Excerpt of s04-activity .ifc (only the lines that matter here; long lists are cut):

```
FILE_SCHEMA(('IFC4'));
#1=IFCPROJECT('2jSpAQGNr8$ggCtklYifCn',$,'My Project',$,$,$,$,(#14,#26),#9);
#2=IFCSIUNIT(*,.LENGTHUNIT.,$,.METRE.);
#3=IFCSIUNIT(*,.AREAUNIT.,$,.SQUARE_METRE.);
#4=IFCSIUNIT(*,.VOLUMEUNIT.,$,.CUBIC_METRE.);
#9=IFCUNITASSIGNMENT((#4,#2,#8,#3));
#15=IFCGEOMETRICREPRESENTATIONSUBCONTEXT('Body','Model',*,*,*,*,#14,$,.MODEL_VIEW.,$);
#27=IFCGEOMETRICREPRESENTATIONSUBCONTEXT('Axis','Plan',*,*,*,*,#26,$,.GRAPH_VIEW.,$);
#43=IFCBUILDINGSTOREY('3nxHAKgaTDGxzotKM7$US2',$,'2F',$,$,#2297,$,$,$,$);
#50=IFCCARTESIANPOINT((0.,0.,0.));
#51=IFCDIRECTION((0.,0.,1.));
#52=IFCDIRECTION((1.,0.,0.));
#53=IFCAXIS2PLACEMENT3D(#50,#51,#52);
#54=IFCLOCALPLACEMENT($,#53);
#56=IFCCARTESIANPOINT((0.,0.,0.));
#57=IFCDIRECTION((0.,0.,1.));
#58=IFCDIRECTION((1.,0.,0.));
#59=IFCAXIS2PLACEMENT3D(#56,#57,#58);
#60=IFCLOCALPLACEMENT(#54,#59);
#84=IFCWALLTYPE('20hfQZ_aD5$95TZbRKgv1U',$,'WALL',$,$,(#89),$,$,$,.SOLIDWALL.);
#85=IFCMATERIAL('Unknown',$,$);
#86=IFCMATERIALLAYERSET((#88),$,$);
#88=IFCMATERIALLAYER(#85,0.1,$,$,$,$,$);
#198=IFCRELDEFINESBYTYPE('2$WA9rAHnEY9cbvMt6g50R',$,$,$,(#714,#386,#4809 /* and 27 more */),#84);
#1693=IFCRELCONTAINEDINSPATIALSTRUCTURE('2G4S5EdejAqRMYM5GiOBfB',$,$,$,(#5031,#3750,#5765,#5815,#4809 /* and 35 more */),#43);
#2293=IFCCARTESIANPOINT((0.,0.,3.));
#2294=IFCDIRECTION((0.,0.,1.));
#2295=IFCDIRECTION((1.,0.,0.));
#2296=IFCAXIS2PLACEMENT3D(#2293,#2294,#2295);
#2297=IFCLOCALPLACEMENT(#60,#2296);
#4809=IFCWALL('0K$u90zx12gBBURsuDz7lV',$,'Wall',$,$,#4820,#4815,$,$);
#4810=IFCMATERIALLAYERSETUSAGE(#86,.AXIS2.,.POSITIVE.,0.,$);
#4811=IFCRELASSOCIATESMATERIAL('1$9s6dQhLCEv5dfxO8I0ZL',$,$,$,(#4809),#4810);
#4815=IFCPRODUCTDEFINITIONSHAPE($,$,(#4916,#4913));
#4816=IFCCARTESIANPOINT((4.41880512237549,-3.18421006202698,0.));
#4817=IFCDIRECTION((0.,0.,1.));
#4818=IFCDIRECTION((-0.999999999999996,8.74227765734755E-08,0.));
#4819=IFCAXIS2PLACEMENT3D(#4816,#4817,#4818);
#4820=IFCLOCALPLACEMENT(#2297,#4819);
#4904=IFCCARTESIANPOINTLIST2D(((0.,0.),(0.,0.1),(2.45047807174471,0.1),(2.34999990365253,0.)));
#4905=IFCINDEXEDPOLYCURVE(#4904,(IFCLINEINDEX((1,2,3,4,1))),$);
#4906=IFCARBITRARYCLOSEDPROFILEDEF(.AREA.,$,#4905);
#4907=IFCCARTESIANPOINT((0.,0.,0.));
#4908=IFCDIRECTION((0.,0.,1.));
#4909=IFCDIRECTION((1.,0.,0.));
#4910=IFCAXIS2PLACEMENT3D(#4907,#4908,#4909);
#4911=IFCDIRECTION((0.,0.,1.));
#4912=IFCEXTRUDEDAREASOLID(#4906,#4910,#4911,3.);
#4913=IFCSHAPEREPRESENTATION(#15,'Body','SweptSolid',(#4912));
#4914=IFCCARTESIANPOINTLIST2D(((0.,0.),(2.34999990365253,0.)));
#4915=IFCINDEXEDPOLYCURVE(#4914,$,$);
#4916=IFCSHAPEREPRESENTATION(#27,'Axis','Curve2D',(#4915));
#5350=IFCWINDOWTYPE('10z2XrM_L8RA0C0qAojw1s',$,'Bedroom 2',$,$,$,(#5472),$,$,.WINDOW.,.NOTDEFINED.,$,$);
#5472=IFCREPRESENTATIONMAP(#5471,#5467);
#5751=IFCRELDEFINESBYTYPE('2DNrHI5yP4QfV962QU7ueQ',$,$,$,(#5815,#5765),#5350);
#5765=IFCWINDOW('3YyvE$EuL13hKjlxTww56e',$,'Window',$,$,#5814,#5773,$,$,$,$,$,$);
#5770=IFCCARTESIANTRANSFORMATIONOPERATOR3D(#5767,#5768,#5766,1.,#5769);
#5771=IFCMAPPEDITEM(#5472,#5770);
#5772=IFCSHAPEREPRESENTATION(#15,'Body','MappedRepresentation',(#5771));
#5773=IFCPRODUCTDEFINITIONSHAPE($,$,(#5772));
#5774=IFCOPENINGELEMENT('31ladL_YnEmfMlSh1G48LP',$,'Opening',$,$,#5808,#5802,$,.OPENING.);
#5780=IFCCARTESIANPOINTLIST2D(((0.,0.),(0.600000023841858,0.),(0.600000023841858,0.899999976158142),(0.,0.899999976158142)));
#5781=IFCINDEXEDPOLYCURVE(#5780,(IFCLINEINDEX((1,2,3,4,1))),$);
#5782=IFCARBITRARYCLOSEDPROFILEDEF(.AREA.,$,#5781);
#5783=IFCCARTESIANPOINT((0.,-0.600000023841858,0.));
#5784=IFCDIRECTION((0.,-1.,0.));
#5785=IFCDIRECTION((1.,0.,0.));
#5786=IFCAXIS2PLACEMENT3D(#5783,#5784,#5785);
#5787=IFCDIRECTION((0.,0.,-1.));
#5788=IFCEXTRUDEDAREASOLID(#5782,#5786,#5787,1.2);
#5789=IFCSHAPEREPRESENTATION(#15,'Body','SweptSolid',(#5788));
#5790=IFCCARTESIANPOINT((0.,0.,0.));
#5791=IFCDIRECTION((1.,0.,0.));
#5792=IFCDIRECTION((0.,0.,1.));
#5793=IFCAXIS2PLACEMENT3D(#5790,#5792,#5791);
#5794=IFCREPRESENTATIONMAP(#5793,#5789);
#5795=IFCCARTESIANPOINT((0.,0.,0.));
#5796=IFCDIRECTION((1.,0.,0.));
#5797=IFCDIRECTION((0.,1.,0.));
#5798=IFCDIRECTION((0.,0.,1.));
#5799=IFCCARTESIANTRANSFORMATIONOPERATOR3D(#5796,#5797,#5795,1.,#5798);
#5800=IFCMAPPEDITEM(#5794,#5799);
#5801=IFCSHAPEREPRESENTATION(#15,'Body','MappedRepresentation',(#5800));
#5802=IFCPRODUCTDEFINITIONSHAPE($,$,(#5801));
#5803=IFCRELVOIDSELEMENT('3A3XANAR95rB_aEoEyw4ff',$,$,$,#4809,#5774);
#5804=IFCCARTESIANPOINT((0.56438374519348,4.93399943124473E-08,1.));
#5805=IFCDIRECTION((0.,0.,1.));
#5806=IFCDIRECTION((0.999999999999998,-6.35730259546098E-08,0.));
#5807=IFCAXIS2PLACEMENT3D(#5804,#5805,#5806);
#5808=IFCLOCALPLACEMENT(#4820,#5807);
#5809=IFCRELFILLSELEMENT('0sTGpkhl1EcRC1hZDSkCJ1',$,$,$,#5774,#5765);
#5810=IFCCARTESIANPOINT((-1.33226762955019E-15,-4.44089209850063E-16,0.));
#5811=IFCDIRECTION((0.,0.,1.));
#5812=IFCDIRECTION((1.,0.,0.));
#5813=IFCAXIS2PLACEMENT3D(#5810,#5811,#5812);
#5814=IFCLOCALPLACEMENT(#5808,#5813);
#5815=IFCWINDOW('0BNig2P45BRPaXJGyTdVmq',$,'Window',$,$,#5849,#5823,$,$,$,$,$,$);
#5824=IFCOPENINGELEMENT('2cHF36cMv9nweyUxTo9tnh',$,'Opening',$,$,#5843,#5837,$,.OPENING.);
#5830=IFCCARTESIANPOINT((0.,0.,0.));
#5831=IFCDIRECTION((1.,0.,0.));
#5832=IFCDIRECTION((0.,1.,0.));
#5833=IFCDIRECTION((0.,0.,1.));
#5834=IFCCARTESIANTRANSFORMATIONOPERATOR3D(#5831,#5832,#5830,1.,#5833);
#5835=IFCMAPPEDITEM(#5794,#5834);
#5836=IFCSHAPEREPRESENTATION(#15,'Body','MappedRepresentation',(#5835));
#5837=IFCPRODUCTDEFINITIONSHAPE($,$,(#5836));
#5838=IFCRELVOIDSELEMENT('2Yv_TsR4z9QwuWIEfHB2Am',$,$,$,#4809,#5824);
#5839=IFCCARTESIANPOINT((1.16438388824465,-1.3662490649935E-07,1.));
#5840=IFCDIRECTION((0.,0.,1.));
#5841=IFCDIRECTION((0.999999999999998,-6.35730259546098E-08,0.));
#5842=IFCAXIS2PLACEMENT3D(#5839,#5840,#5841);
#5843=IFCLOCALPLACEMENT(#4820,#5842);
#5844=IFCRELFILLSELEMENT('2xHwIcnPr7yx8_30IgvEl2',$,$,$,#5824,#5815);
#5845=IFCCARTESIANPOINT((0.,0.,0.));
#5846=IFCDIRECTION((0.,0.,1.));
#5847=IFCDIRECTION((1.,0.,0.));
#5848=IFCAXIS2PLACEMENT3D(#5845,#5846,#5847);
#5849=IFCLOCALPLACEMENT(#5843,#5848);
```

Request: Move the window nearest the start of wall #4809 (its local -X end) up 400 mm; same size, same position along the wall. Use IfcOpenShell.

```python
import numpy as np
import ifcopenshell
import ifcopenshell.api.geometry
import ifcopenshell.util.placement
import ifcopenshell.util.unit

model = ifcopenshell.open("s04-activity .ifc")
unit_scale = ifcopenshell.util.unit.calculate_unit_scale(model)

window = model.by_guid("3YyvE$EuL13hKjlxTww56e")
opening = window.FillsVoids[0].RelatingOpeningElement
dz = 0.4 / unit_scale

shift = np.array([0.0, 0.0, dz])
# The window is placed relative to its opening, so it follows when the opening moves.
matrix = ifcopenshell.util.placement.get_local_placement(opening.ObjectPlacement)
matrix[:3, 3] += shift
ifcopenshell.api.geometry.edit_object_placement(
    model, product=opening, matrix=matrix, is_si=False, should_transform_children=True
)

print(f"moved by {dz * unit_scale:+.3f} m")

model.write("s04-activity _edited.ifc")
```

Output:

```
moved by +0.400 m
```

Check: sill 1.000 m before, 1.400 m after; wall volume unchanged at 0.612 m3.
